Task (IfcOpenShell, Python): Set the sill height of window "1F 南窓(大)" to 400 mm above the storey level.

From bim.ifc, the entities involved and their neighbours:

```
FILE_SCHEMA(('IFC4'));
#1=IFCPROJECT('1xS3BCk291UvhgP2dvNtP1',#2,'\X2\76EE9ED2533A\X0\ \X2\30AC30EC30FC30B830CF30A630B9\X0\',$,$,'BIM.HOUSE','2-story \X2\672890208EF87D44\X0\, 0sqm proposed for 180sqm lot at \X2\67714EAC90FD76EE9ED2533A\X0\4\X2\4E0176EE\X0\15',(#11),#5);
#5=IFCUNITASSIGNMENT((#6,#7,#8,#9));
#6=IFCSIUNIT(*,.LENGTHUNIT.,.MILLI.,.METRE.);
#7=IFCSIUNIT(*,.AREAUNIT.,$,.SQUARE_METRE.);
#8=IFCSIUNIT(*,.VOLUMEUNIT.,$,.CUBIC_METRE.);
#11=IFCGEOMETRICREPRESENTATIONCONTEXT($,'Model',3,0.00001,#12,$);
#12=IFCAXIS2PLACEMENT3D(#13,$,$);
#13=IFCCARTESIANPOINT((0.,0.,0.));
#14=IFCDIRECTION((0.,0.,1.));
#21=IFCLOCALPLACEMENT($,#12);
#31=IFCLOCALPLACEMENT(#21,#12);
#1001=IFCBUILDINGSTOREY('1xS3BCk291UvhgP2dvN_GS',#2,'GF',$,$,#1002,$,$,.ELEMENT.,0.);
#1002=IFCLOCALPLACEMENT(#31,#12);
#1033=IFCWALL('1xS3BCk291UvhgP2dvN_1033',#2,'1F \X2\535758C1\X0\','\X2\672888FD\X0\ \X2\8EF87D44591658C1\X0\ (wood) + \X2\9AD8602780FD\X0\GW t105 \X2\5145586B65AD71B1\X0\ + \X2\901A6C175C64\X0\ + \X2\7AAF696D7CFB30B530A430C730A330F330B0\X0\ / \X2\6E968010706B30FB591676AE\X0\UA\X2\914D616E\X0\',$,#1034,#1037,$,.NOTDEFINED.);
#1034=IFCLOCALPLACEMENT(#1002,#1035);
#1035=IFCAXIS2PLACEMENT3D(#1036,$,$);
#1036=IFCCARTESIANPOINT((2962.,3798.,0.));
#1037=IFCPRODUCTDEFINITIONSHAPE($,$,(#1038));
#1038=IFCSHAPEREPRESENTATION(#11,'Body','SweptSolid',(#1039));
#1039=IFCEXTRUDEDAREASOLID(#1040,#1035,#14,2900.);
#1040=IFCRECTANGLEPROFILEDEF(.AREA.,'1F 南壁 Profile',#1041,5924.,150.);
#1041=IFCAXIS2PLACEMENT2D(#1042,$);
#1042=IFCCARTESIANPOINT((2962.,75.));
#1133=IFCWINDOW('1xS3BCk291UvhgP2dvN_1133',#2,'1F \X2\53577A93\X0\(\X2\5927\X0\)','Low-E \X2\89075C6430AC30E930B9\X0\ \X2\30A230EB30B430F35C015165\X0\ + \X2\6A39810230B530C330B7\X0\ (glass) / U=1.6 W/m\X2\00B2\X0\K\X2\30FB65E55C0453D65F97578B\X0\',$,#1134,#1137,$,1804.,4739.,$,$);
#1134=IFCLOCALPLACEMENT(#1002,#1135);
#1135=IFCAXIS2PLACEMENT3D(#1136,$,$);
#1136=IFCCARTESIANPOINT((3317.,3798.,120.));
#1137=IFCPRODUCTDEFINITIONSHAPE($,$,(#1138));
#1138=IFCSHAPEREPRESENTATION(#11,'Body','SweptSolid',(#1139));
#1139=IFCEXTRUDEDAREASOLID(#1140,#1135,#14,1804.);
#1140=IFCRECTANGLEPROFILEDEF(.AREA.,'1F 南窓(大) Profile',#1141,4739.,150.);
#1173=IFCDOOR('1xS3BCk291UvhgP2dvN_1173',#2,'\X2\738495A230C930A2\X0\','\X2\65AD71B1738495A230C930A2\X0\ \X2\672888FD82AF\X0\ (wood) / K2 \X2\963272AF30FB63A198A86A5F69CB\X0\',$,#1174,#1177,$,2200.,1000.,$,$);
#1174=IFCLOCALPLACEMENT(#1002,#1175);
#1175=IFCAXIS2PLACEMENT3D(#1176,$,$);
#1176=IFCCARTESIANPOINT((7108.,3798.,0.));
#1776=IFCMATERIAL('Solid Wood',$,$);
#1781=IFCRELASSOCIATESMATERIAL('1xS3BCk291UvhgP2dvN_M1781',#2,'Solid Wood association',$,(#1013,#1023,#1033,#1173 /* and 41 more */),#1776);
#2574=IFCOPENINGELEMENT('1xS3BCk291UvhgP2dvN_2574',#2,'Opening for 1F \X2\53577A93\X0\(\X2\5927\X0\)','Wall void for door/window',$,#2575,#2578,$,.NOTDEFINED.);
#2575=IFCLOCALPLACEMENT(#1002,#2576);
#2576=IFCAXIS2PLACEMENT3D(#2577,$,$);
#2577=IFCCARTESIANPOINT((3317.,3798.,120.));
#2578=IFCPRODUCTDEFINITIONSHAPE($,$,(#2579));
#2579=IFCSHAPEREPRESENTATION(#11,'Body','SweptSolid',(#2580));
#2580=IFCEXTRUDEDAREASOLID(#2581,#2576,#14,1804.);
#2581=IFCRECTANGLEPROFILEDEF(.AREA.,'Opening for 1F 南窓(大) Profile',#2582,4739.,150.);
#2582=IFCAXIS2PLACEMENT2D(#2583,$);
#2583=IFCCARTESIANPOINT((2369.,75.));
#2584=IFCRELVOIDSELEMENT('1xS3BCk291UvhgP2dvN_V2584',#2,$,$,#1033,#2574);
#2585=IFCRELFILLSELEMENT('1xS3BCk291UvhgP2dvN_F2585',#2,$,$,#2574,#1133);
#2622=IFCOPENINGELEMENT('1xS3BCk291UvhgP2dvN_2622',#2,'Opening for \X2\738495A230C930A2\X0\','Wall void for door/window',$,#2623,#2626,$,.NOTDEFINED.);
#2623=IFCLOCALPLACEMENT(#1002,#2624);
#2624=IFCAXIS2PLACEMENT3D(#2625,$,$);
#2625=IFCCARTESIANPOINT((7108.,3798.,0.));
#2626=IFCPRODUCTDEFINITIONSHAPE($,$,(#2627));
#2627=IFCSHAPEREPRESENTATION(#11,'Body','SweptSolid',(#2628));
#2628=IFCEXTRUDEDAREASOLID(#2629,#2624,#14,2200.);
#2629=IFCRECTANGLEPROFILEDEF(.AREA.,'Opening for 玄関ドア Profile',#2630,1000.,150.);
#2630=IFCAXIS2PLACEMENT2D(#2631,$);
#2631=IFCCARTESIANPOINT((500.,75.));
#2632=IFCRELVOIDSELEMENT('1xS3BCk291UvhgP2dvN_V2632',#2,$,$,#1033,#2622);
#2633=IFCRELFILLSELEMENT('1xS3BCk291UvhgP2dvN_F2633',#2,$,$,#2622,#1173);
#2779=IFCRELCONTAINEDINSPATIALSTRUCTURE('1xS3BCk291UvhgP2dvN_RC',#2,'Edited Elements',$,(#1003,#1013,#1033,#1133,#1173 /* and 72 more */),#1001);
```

```python
import numpy as np
import ifcopenshell
import ifcopenshell.api.geometry
import ifcopenshell.geom
import ifcopenshell.util.element
import ifcopenshell.util.placement
import ifcopenshell.util.shape
import ifcopenshell.util.unit

model = ifcopenshell.open("bim.ifc")
unit_scale = ifcopenshell.util.unit.calculate_unit_scale(model)

window = model.by_guid("1xS3BCk291UvhgP2dvN_1133")
opening = window.FillsVoids[0].RelatingOpeningElement
storey = ifcopenshell.util.element.get_container(window, ifc_class="IfcBuildingStorey")
level = ifcopenshell.util.placement.get_local_placement(storey.ObjectPlacement)[2, 3]

# The opening's origin need not be at the sill, so measure its lowest point.
shape = ifcopenshell.geom.create_shape(ifcopenshell.geom.settings(), opening)
bottom = ifcopenshell.util.shape.get_shape_bottom_elevation(shape, shape.geometry) / unit_scale
dz = level + 400.0 - bottom

shift = np.array([0.0, 0.0, dz])
# The window is not placed relative to its opening, so move both.
for product in (opening, window):
    matrix = ifcopenshell.util.placement.get_local_placement(product.ObjectPlacement)
    matrix[:3, 3] += shift
    ifcopenshell.api.geometry.edit_object_placement(model, product=product, matrix=matrix, is_si=False)

print(f"moved by {dz * unit_scale:+.3f} m")

model.write("bim-out.ifc")
```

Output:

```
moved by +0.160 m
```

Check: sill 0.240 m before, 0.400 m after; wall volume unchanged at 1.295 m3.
